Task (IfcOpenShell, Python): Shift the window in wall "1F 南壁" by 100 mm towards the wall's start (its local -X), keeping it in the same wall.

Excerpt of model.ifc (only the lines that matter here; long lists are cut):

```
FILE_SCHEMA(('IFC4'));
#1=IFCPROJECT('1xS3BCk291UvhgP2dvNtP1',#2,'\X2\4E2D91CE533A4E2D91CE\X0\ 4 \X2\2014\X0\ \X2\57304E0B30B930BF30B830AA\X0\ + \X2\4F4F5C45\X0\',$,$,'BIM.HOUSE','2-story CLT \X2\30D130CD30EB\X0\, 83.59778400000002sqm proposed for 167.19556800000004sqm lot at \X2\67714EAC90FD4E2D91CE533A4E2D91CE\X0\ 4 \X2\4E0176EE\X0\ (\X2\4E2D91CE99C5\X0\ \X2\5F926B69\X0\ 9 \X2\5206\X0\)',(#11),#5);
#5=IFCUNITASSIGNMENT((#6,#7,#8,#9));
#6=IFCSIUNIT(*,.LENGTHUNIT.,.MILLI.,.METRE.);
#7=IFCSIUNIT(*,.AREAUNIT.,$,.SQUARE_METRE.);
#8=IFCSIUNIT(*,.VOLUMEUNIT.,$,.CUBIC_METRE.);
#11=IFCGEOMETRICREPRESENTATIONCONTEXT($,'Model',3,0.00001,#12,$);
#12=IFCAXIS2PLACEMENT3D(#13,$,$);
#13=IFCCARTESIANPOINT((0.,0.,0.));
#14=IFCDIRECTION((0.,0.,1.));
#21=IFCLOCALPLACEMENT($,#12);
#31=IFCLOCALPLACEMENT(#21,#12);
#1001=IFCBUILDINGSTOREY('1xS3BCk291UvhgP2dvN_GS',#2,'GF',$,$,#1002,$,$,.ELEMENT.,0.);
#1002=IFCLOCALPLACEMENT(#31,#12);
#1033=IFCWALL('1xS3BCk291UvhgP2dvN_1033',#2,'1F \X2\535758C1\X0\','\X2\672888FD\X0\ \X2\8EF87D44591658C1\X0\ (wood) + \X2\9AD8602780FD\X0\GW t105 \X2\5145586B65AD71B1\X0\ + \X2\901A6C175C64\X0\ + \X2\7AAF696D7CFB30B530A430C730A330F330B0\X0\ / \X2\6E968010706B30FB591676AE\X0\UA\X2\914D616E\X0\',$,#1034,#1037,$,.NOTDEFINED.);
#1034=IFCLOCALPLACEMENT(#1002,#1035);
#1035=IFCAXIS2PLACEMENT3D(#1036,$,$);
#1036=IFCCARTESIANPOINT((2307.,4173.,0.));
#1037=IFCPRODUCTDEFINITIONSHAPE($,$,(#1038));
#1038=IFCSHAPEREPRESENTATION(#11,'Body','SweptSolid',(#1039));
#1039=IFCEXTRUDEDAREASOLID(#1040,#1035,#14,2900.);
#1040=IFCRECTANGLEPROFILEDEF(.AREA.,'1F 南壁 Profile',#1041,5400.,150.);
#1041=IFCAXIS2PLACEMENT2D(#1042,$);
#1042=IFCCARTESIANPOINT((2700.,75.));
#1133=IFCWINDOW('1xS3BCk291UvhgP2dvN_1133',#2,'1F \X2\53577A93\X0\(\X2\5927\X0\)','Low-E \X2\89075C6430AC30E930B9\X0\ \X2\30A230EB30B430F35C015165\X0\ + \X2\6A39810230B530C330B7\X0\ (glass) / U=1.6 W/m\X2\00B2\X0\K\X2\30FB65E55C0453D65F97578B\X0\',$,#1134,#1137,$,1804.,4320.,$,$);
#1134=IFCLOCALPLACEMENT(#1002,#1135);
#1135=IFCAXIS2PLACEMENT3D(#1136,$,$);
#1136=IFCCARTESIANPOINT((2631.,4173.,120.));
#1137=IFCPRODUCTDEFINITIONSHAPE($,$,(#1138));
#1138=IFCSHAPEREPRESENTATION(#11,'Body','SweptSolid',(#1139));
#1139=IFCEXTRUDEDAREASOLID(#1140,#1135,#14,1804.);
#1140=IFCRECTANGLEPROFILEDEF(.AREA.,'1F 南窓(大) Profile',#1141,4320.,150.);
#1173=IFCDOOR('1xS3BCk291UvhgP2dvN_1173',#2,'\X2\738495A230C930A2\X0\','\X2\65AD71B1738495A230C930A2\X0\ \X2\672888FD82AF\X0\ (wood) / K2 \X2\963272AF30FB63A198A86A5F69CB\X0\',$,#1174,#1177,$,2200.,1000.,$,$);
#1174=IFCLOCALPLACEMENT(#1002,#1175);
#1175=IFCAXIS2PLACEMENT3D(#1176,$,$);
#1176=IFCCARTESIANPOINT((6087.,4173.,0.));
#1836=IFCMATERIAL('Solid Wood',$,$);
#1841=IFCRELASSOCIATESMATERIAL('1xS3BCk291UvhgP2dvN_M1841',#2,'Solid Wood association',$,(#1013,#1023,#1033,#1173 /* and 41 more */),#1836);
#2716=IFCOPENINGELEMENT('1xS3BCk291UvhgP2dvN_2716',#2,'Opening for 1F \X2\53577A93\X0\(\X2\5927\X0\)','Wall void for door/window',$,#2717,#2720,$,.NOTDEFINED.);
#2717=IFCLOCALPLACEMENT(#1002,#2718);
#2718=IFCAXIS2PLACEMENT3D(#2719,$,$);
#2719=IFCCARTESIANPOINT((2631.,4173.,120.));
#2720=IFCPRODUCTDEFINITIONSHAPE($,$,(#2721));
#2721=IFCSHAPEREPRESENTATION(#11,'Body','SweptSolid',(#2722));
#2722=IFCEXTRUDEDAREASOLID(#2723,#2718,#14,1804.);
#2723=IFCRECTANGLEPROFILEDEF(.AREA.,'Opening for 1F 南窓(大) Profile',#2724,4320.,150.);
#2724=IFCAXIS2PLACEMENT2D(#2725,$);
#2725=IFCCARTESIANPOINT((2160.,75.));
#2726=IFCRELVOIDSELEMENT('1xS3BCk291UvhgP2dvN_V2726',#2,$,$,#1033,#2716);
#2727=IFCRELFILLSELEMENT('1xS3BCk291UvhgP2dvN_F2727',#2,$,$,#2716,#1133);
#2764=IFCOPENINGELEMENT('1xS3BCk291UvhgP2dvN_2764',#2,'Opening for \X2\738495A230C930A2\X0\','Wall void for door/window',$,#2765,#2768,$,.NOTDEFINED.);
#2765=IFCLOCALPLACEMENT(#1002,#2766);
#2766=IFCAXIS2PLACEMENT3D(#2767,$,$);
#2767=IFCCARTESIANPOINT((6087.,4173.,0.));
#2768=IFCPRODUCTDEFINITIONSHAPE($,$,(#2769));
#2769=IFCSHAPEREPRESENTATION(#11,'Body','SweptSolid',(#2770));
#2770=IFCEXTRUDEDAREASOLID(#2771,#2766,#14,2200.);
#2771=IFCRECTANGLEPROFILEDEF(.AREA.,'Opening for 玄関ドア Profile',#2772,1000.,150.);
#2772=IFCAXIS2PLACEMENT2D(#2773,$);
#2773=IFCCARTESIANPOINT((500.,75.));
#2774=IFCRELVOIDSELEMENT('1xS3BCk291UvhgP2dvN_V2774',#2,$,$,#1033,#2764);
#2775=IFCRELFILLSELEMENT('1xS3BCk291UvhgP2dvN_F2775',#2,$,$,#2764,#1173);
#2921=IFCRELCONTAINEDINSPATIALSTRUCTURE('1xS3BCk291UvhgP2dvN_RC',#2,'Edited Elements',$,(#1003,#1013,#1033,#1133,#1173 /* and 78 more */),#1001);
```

```python
import ifcopenshell
import ifcopenshell.api.geometry
import ifcopenshell.util.placement
import ifcopenshell.util.unit

model = ifcopenshell.open("model.ifc")
unit_scale = ifcopenshell.util.unit.calculate_unit_scale(model)

window = model.by_guid("1xS3BCk291UvhgP2dvN_1133")
opening = window.FillsVoids[0].RelatingOpeningElement
wall = opening.VoidsElements[0].RelatingBuildingElement

wall_matrix = ifcopenshell.util.placement.get_local_placement(wall.ObjectPlacement)
shift = wall_matrix[:3, 0] * -0.1 / unit_scale
before = ifcopenshell.util.placement.get_local_placement(window.ObjectPlacement)[:3, 3].copy()

# The window is not placed relative to its opening, so move both.
for product in (opening, window):
    matrix = ifcopenshell.util.placement.get_local_placement(product.ObjectPlacement)
    matrix[:3, 3] += shift
    ifcopenshell.api.geometry.edit_object_placement(model, product=product, matrix=matrix, is_si=False)

after = ifcopenshell.util.placement.get_local_placement(window.ObjectPlacement)[:3, 3]
print("window moved by", (after - before).round(3) + 0.0)

model.write("model-out.ifc")
```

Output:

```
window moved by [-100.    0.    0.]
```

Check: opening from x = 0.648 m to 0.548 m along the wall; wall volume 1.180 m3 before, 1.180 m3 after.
